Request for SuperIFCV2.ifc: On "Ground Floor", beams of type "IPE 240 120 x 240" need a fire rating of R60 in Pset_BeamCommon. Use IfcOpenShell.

First a look at what the model holds.

```python
import ifcopenshell
import ifcopenshell.util.element

model = ifcopenshell.open("SuperIFCV2.ifc")
print(model.schema)
storey = next(s for s in model.by_type("IfcBuildingStorey") if s.Name == "Ground Floor")
beams = [e for e in ifcopenshell.util.element.get_decomposition(storey) if e.is_a("IfcBeam")]
seen = {}
for e in beams:
    element_type = ifcopenshell.util.element.get_type(e)
    key = (element_type.Name if element_type != e and element_type else None, ifcopenshell.util.element.get_pset(e, "Pset_BeamCommon", "FireRating"))
    seen[key] = seen.get(key, 0) + 1
for (name, value), count in sorted(seen.items(), key=str):
    print(count, "x", name, "|", value)
```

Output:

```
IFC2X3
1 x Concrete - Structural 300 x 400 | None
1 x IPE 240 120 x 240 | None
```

```python
import ifcopenshell
import ifcopenshell.api.pset
import ifcopenshell.util.element

model = ifcopenshell.open("SuperIFCV2.ifc")

storey = next(s for s in model.by_type("IfcBuildingStorey") if s.Name == "Ground Floor")
beams = [e for e in ifcopenshell.util.element.get_decomposition(storey) if e.is_a("IfcBeam")]

count = 0
for e in beams:
    element_type = ifcopenshell.util.element.get_type(e)
    if element_type in (None, e) or element_type.Name != "IPE 240 120 x 240":
        continue
    # add_pset returns the element's existing set when there is one.
    pset = ifcopenshell.api.pset.add_pset(model, product=e, name="Pset_BeamCommon")
    ifcopenshell.api.pset.edit_pset(model, pset=pset, properties={"FireRating": "R60"})
    count += 1

print(count, "beams updated")

model.write("SuperIFCV2_v2.ifc")
```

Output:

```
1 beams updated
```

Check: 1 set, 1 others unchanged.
